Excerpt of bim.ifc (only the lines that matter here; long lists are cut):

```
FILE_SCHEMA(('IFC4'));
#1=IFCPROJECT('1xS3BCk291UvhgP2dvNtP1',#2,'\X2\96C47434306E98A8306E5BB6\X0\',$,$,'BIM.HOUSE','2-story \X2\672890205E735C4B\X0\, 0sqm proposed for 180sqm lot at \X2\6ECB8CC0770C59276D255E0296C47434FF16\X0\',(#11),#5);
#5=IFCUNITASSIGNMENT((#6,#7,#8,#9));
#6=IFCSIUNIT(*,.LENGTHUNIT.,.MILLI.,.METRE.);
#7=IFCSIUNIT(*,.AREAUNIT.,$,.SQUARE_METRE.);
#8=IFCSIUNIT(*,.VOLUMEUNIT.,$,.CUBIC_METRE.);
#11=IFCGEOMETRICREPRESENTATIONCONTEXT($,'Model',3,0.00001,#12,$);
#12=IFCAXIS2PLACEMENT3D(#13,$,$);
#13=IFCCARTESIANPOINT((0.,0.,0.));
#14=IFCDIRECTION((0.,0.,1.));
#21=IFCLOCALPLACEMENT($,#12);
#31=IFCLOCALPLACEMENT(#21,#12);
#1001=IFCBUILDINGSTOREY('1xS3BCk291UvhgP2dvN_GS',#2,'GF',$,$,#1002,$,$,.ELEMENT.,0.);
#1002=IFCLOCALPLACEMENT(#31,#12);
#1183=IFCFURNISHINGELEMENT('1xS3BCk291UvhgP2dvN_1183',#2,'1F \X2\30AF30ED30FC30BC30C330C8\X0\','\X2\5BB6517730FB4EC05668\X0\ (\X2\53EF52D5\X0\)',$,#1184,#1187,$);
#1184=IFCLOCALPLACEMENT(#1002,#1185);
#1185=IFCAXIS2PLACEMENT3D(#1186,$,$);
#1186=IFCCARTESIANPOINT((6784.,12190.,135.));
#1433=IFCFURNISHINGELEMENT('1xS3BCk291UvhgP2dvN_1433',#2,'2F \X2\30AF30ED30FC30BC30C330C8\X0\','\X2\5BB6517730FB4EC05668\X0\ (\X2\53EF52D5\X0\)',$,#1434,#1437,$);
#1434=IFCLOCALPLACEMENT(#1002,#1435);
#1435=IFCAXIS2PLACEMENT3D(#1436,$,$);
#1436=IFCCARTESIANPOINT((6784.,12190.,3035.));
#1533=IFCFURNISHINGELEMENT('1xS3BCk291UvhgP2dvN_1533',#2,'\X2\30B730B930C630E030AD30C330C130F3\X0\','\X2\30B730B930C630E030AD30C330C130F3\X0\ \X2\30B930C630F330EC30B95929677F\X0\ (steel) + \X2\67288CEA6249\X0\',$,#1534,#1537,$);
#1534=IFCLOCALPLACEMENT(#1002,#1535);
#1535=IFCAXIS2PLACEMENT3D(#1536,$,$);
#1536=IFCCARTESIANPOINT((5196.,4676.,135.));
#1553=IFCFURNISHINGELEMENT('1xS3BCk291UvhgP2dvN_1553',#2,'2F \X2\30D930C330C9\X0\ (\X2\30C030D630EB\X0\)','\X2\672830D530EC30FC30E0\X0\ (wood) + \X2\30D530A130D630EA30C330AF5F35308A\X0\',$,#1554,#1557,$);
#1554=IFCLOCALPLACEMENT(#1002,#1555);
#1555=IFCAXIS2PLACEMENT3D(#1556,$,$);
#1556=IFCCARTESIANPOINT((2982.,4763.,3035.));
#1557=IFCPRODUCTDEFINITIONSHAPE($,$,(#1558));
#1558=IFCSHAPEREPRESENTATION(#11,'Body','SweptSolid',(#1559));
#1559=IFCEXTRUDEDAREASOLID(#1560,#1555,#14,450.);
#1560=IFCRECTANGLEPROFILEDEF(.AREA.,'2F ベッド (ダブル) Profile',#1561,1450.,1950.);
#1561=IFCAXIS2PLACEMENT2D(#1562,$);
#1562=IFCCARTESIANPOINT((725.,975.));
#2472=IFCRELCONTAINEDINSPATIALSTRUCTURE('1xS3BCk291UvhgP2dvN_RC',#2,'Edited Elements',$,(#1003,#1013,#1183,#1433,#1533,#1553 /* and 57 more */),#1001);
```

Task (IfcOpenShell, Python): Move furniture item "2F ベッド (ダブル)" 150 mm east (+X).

```python
import ifcopenshell
import ifcopenshell.api.geometry
import ifcopenshell.util.placement
import ifcopenshell.util.unit

model = ifcopenshell.open("bim.ifc")
unit_scale = ifcopenshell.util.unit.calculate_unit_scale(model)

item = model.by_guid("1xS3BCk291UvhgP2dvN_1553")
matrix = ifcopenshell.util.placement.get_local_placement(item.ObjectPlacement)
matrix[0, 3] += 0.15 / unit_scale
ifcopenshell.api.geometry.edit_object_placement(model, product=item, matrix=matrix, is_si=False)

print(ifcopenshell.util.placement.get_local_placement(item.ObjectPlacement).round(3) + 0.0)

model.write("bim_edited.ifc")
```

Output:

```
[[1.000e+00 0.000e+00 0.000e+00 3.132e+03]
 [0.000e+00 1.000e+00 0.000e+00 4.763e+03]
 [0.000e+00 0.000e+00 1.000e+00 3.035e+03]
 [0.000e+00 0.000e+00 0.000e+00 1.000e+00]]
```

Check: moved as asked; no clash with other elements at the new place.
